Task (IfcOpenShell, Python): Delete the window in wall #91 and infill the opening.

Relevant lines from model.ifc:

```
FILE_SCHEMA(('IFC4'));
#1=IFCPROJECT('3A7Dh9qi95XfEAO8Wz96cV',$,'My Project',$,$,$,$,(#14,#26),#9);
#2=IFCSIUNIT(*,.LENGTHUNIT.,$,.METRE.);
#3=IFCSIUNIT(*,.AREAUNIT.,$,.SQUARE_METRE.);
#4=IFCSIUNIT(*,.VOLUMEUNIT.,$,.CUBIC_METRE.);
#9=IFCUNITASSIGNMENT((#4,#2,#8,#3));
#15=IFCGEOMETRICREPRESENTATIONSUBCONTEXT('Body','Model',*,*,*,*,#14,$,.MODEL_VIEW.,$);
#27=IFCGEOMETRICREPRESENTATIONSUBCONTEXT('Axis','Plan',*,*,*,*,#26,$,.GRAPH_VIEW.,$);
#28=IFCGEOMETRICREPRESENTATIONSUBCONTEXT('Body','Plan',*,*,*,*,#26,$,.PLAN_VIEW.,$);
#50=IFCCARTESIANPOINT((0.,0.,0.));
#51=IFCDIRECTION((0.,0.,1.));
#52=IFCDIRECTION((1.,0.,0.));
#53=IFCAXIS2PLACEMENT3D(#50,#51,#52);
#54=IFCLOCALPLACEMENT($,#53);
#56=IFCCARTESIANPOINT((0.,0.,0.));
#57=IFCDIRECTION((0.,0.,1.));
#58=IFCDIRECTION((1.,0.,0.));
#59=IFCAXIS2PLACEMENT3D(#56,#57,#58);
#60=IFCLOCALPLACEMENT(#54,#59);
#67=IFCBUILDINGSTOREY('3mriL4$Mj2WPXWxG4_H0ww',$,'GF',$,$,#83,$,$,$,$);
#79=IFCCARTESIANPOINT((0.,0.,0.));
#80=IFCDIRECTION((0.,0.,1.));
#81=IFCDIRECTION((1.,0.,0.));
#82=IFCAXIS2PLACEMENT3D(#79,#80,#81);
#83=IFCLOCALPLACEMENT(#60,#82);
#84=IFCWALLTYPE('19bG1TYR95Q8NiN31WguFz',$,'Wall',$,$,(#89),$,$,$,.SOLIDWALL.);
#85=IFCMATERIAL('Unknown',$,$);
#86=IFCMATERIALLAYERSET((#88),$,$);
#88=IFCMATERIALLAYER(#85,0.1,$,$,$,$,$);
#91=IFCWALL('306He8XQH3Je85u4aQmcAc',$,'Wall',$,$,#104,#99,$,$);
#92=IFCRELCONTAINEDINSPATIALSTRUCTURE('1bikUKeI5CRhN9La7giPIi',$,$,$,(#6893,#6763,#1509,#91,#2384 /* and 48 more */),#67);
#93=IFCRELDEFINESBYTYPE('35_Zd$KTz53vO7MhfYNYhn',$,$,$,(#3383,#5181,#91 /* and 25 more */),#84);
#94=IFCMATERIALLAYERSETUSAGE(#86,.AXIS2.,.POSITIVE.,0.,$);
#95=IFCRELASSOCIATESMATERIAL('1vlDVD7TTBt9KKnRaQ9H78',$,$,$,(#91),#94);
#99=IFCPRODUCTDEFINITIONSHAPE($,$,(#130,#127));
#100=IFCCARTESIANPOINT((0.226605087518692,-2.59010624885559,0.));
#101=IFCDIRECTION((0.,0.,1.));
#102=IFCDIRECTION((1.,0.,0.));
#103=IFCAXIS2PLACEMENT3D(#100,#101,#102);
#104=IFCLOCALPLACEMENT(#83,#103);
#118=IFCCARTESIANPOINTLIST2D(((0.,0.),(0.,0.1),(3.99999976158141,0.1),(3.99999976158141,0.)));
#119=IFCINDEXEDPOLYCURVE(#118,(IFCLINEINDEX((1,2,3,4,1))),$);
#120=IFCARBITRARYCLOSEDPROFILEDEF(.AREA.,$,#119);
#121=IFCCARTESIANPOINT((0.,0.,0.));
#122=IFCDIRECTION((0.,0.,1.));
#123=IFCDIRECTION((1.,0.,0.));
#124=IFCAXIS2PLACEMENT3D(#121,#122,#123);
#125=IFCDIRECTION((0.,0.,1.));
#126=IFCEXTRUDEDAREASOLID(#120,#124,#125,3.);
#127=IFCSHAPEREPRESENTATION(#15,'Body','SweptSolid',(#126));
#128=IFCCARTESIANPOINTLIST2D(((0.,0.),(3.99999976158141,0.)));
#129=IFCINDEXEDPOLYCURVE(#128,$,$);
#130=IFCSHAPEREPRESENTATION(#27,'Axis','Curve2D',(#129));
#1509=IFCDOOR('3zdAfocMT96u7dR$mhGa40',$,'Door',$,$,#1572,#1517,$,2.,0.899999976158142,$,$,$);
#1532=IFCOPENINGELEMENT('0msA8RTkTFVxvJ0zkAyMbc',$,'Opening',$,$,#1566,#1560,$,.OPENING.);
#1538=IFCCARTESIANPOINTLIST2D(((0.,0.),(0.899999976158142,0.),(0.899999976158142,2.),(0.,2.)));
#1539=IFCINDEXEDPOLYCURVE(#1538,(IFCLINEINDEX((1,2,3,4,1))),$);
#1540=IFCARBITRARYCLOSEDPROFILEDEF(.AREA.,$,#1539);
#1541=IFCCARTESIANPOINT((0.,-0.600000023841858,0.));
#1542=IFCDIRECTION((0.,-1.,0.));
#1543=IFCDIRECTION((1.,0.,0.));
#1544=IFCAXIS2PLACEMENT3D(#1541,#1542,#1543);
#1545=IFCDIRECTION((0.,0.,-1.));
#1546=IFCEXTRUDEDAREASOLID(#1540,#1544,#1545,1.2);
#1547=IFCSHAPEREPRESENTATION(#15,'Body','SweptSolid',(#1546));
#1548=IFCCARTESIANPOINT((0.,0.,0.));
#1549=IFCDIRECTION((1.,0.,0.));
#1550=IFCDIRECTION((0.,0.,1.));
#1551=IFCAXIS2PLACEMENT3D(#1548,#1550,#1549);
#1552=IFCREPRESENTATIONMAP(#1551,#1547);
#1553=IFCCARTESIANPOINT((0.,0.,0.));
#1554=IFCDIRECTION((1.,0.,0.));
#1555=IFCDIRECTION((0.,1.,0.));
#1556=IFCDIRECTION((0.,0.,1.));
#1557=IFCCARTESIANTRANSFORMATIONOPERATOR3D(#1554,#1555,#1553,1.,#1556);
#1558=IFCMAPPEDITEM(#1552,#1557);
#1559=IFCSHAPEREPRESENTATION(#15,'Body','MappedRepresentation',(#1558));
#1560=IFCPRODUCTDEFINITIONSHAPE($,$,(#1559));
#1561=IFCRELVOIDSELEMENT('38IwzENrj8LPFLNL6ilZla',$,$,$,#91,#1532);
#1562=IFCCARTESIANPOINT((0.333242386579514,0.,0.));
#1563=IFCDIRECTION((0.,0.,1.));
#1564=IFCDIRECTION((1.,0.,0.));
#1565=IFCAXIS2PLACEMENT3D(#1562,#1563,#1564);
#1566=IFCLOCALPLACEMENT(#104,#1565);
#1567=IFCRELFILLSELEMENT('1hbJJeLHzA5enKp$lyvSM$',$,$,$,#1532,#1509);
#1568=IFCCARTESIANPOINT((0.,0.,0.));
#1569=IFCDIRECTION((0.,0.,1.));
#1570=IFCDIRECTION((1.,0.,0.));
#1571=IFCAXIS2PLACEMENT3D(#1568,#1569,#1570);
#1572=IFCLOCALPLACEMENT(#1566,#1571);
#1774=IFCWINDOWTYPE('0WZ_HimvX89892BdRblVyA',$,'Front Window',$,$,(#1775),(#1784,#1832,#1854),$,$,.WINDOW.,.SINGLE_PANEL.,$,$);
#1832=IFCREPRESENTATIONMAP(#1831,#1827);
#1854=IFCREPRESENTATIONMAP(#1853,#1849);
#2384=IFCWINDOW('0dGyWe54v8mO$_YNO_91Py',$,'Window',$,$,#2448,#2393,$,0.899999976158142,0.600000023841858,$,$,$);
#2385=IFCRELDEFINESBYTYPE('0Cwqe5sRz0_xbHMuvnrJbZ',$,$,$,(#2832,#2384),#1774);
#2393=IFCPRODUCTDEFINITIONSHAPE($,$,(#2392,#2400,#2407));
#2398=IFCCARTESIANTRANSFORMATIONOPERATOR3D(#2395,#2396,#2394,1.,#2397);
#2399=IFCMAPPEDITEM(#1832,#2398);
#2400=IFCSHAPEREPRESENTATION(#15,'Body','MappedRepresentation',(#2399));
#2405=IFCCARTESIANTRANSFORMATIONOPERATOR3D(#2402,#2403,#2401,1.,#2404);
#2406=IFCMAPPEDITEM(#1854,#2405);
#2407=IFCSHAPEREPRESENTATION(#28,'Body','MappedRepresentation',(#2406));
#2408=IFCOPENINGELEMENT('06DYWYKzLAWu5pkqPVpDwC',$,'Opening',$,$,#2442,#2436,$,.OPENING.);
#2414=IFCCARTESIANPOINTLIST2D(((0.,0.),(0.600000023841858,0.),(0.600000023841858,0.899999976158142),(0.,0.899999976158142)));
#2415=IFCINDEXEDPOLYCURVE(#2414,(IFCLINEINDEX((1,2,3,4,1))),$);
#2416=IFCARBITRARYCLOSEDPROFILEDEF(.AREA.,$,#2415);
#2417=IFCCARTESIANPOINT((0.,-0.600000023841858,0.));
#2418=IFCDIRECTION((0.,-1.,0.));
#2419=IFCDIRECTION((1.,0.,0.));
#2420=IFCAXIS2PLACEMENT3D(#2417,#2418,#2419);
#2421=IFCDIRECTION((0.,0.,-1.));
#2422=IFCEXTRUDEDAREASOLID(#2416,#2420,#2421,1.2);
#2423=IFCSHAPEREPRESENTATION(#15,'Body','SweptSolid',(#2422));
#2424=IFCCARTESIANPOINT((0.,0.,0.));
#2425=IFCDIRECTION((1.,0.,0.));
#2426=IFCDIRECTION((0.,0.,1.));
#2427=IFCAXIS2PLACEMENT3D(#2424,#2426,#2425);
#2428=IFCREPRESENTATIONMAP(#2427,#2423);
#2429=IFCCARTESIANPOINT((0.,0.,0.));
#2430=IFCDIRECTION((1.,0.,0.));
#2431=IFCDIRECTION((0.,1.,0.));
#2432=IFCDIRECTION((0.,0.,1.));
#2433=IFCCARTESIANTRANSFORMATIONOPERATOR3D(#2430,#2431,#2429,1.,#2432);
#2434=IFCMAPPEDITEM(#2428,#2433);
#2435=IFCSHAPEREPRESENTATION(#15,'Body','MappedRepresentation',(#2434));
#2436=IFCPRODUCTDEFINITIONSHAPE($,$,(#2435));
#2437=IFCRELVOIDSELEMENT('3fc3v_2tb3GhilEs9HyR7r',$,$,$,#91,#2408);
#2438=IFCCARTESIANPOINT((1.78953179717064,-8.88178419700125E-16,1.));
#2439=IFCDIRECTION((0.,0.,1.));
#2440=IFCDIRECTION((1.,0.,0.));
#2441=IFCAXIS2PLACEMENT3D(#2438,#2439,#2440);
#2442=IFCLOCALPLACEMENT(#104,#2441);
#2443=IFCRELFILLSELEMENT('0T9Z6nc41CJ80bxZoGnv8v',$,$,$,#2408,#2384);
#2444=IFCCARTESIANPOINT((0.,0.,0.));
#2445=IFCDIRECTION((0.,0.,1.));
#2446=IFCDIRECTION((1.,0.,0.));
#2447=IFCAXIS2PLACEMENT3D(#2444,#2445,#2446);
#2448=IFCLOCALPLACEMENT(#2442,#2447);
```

```python
import ifcopenshell
import ifcopenshell.api.feature
import ifcopenshell.api.root
import ifcopenshell.geom
import ifcopenshell.util.shape

model = ifcopenshell.open("model.ifc")
settings = ifcopenshell.geom.settings()


def volume(element):
    """Net volume in cubic metres, openings subtracted."""
    shape = ifcopenshell.geom.create_shape(settings, element)
    return ifcopenshell.util.shape.get_volume(shape.geometry)


window = model.by_guid("0dGyWe54v8mO$_YNO_91Py")
opening = window.FillsVoids[0].RelatingOpeningElement
wall = opening.VoidsElements[0].RelatingBuildingElement
before = volume(wall)

ifcopenshell.api.root.remove_product(model, product=window)
ifcopenshell.api.feature.remove_feature(model, feature=opening)

after = volume(wall)

print(f"wall volume {before:.3f} -> {after:.3f} m3")

model.write("model-out.ifc")
```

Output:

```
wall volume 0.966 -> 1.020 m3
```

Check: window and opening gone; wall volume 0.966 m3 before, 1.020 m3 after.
